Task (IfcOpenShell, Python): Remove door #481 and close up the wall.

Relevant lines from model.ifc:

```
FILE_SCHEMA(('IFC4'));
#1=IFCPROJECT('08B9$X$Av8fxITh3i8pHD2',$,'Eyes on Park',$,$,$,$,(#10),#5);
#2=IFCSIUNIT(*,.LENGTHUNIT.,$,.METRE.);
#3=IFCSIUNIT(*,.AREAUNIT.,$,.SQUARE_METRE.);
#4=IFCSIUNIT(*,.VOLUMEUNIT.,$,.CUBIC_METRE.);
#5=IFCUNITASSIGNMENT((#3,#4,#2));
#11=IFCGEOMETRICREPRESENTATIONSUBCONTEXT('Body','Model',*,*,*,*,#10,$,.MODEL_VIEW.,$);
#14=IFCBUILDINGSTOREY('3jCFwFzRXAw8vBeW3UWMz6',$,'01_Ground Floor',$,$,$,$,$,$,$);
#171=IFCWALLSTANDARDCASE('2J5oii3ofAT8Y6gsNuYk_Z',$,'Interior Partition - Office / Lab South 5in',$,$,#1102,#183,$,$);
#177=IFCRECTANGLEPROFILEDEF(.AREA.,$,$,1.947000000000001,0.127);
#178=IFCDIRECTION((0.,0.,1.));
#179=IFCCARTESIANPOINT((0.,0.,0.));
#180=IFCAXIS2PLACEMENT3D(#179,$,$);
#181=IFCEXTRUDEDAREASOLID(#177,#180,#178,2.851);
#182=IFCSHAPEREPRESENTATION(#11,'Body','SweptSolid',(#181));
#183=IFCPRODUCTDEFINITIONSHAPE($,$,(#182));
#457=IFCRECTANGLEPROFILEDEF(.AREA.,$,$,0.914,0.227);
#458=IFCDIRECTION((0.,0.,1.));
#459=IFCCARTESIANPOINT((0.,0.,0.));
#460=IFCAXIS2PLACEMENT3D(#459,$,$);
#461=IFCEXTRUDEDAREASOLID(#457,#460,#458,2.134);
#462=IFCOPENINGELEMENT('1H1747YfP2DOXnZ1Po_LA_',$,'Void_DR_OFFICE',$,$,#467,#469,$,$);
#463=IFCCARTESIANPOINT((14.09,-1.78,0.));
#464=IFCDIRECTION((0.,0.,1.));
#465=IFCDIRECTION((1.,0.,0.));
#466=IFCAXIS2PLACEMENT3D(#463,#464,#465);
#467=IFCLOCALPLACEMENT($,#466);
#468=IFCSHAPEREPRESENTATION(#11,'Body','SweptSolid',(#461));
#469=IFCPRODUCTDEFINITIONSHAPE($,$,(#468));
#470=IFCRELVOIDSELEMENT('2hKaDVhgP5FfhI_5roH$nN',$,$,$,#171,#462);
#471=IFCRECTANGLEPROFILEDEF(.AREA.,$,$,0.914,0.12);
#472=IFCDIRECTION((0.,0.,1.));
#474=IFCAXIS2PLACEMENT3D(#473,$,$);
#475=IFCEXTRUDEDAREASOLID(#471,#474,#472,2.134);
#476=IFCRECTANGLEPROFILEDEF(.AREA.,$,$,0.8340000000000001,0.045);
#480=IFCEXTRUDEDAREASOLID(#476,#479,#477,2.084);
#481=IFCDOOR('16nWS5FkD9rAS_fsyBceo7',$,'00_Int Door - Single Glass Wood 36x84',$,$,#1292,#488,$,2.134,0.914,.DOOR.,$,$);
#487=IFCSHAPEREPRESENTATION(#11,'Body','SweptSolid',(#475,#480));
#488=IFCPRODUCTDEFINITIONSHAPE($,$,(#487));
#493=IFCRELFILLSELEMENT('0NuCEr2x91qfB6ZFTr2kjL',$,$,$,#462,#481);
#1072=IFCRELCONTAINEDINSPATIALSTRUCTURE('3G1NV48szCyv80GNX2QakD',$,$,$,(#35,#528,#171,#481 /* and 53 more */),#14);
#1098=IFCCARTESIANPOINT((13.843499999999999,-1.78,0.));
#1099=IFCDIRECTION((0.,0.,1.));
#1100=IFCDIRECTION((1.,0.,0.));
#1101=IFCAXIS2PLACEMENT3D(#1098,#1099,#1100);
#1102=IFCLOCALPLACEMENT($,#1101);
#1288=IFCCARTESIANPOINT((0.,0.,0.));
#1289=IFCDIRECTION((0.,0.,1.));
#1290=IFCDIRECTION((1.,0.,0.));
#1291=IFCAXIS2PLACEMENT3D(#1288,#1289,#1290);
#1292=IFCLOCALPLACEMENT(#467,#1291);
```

```python
import ifcopenshell
import ifcopenshell.api.feature
import ifcopenshell.api.root
import ifcopenshell.geom
import ifcopenshell.util.shape

model = ifcopenshell.open("model.ifc")
settings = ifcopenshell.geom.settings()


def volume(element):
    """Net volume in cubic metres, openings subtracted."""
    shape = ifcopenshell.geom.create_shape(settings, element)
    return ifcopenshell.util.shape.get_volume(shape.geometry)


door = model.by_guid("16nWS5FkD9rAS_fsyBceo7")
opening = door.FillsVoids[0].RelatingOpeningElement
wall = opening.VoidsElements[0].RelatingBuildingElement
before = volume(wall)

ifcopenshell.api.root.remove_product(model, product=door)
ifcopenshell.api.feature.remove_feature(model, feature=opening)

after = volume(wall)

print(f"wall volume {before:.3f} -> {after:.3f} m3")

model.write("model_v2.ifc")
```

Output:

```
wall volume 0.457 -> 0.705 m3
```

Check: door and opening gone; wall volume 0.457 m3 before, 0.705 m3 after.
